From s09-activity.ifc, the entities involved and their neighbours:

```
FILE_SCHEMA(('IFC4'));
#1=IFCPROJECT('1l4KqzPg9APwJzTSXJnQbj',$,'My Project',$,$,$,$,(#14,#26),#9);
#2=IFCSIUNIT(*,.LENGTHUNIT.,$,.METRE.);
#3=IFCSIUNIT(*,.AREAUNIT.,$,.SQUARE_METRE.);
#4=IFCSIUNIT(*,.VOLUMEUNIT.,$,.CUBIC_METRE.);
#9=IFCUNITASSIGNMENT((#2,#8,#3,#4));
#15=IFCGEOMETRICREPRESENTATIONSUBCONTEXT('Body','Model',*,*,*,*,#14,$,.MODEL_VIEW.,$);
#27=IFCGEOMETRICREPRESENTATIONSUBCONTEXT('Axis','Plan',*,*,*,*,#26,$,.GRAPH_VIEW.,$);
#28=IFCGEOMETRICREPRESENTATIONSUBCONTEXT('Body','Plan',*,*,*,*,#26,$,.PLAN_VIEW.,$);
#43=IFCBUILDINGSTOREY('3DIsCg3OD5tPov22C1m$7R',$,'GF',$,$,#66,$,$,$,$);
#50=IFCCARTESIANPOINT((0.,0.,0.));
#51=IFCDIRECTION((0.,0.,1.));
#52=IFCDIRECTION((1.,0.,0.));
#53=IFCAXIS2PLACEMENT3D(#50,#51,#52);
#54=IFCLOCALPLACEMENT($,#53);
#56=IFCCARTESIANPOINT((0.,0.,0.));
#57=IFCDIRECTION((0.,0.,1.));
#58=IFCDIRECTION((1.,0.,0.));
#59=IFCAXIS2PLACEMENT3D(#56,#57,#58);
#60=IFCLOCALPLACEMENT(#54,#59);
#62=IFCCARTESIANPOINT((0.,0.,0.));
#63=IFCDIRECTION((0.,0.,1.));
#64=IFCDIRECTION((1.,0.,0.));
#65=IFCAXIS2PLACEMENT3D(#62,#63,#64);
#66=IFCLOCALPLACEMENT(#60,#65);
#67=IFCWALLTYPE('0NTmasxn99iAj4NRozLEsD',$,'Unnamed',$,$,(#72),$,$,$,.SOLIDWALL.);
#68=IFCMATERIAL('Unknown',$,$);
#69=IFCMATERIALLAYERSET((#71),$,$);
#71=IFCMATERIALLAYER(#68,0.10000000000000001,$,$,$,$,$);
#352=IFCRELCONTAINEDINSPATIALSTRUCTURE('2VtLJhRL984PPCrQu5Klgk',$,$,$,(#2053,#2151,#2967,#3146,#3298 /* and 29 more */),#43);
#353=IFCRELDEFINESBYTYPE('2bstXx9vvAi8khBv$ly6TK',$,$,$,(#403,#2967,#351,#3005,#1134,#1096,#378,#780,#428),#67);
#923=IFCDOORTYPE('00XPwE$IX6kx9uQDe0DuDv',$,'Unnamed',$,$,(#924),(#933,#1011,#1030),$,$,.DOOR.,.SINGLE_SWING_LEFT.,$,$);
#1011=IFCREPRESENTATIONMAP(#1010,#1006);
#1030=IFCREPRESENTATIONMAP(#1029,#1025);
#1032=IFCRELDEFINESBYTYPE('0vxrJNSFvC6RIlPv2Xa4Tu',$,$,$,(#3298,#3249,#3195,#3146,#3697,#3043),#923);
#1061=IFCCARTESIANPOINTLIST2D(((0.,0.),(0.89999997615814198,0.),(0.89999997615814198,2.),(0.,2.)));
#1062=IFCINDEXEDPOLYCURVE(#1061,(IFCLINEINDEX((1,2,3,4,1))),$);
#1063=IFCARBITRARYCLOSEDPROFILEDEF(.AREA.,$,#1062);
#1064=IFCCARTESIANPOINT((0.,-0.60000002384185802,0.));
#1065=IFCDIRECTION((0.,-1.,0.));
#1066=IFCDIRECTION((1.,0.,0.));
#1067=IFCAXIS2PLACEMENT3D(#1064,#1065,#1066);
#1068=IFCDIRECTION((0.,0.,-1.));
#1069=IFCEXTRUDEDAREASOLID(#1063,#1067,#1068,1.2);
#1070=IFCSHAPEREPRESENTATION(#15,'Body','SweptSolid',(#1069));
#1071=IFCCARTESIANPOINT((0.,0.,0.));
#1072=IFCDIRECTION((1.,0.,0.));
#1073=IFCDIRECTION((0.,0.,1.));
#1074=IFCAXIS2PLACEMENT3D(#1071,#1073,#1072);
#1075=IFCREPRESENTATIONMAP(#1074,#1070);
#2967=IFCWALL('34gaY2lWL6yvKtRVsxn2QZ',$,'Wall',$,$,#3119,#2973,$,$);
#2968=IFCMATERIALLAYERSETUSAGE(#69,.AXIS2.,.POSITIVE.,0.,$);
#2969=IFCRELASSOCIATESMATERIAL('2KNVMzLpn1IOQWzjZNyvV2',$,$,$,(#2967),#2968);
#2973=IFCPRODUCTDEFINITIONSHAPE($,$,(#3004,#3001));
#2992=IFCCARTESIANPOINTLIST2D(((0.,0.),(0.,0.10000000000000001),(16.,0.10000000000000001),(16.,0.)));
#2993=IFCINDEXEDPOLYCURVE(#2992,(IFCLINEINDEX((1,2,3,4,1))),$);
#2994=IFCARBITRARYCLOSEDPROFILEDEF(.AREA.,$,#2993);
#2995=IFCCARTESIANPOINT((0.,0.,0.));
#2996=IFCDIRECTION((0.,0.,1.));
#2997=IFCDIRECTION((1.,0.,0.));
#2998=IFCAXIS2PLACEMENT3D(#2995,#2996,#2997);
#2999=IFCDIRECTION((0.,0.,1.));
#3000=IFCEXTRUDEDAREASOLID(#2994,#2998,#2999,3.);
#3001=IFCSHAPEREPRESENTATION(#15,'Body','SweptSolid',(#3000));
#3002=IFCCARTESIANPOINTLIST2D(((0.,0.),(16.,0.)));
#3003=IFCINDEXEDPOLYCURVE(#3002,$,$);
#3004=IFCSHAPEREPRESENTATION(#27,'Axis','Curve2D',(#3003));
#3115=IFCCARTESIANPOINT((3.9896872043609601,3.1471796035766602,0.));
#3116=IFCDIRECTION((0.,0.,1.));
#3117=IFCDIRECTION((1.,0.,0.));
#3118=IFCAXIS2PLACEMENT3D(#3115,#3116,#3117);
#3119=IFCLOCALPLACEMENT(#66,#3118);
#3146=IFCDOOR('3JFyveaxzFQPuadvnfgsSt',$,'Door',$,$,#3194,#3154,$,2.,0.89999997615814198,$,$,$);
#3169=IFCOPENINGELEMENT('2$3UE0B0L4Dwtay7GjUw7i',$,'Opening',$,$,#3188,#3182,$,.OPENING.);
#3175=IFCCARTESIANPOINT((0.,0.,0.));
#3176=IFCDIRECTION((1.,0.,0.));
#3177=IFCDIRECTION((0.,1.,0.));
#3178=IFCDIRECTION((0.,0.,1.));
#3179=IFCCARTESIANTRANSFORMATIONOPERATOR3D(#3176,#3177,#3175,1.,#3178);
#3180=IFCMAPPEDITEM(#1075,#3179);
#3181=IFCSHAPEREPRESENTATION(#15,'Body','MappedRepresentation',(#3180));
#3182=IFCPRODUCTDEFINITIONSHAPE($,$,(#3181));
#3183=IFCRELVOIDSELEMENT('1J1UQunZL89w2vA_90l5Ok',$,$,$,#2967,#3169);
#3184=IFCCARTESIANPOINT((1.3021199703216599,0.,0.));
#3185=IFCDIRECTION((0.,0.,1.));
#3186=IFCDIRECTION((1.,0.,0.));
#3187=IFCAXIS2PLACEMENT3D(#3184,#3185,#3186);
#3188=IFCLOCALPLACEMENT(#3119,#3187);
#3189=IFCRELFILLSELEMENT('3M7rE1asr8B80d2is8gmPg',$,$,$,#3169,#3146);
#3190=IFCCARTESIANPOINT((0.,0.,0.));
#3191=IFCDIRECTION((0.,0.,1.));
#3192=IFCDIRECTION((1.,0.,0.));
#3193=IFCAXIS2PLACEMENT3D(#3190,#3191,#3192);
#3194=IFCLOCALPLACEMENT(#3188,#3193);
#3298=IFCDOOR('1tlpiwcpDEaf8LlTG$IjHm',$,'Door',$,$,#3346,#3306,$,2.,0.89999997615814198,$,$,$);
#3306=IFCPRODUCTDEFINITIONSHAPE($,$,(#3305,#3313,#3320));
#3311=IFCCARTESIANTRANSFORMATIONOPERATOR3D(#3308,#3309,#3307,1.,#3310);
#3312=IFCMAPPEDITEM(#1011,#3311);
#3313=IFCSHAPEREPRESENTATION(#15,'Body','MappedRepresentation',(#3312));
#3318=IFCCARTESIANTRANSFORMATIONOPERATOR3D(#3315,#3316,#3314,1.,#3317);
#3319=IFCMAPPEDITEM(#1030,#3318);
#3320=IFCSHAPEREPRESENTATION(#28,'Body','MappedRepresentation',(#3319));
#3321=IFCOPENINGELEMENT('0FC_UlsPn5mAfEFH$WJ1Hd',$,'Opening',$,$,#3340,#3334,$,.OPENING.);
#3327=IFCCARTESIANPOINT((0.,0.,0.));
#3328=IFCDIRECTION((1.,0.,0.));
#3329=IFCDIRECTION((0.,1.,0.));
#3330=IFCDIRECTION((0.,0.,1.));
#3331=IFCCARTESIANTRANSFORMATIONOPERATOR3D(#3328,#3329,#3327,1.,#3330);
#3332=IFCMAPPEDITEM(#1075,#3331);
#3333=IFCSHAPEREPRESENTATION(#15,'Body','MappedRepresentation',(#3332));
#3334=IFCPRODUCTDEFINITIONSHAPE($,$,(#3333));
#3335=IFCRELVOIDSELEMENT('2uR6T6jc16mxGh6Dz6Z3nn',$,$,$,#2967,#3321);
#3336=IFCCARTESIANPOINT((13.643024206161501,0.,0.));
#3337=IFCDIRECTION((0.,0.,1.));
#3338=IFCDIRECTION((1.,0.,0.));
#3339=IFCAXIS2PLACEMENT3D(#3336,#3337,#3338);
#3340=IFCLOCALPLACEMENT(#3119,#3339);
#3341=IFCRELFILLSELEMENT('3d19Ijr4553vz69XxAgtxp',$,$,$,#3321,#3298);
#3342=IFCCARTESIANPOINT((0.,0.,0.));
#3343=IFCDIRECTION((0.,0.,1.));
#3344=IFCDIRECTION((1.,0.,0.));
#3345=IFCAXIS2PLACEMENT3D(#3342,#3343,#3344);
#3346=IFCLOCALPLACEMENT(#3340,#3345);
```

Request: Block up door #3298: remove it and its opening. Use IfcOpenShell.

```python
import ifcopenshell
import ifcopenshell.api.feature
import ifcopenshell.api.root
import ifcopenshell.geom
import ifcopenshell.util.shape

model = ifcopenshell.open("s09-activity.ifc")
settings = ifcopenshell.geom.settings()


def volume(element):
    """Net volume in cubic metres, openings subtracted."""
    shape = ifcopenshell.geom.create_shape(settings, element)
    return ifcopenshell.util.shape.get_volume(shape.geometry)


door = model.by_guid("1tlpiwcpDEaf8LlTG$IjHm")
opening = door.FillsVoids[0].RelatingOpeningElement
wall = opening.VoidsElements[0].RelatingBuildingElement
before = volume(wall)

ifcopenshell.api.root.remove_product(model, product=door)
ifcopenshell.api.feature.remove_feature(model, feature=opening)

after = volume(wall)

print(f"wall volume {before:.3f} -> {after:.3f} m3")

model.write("s09-activity_edited.ifc")
```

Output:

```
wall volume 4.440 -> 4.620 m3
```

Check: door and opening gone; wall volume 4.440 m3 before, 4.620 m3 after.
